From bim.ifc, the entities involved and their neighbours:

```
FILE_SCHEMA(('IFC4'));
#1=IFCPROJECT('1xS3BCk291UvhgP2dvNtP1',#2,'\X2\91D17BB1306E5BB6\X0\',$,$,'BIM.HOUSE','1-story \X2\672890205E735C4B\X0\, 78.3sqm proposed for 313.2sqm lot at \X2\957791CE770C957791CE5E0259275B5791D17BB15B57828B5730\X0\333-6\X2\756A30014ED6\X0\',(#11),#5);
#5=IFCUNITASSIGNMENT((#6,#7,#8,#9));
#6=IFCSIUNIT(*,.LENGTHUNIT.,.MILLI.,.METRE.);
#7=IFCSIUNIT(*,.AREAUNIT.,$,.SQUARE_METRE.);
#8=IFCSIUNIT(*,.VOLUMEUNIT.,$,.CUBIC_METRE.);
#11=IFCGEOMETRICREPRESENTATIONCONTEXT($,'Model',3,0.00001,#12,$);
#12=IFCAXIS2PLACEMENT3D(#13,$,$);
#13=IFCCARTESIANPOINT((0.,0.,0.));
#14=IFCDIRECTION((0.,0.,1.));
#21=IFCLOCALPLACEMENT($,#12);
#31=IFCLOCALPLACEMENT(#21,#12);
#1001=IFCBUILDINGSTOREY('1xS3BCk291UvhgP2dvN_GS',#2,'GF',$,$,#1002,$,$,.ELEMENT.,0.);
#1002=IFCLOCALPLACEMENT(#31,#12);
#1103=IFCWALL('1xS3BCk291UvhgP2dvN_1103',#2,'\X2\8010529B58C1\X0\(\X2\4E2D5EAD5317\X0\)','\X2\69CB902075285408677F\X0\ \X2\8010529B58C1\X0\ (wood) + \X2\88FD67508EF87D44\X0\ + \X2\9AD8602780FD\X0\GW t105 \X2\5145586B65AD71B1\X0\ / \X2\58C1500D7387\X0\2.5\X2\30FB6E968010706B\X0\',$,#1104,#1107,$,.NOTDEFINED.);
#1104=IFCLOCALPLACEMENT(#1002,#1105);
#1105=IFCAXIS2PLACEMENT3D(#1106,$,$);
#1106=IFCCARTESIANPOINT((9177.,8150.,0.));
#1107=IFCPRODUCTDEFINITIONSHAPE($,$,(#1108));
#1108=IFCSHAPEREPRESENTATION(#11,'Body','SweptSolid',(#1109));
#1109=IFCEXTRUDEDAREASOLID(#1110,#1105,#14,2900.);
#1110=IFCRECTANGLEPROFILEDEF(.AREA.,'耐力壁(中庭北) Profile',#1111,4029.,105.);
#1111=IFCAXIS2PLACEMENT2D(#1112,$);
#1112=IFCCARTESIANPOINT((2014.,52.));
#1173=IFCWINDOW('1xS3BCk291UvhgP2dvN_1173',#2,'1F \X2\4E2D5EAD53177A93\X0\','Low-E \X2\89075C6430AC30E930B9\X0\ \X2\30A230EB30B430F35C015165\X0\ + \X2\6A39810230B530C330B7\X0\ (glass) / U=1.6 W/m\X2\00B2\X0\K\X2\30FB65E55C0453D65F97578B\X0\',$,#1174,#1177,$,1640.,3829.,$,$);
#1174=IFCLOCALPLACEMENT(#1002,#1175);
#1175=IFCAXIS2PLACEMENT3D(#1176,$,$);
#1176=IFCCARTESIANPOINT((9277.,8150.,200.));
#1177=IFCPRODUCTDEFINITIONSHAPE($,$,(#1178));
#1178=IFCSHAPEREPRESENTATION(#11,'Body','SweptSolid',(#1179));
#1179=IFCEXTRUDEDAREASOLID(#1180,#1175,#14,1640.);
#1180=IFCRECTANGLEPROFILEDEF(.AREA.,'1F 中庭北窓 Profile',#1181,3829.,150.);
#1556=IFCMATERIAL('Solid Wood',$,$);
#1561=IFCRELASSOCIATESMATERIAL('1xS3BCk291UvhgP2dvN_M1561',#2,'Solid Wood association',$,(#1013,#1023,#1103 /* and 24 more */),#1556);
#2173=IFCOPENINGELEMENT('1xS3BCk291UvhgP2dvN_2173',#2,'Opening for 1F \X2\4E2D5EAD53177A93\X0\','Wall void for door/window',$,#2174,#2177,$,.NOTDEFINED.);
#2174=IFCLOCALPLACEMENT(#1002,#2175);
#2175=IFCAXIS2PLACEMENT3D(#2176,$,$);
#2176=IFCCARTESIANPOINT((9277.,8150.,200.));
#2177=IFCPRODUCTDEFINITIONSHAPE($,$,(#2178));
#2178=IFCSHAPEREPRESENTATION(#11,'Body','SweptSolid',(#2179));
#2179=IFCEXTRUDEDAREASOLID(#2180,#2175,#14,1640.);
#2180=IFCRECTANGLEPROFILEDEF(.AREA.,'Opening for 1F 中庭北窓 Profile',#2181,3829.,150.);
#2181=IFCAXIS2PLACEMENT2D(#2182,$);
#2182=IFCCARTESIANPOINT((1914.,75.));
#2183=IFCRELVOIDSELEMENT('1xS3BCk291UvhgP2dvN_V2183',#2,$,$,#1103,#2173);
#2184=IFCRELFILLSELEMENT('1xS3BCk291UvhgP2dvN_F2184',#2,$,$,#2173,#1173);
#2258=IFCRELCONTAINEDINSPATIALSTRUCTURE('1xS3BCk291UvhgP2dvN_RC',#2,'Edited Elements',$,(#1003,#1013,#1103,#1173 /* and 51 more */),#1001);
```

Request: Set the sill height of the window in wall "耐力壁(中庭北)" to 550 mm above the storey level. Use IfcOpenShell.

```python
import numpy as np
import ifcopenshell
import ifcopenshell.api.geometry
import ifcopenshell.geom
import ifcopenshell.util.element
import ifcopenshell.util.placement
import ifcopenshell.util.shape
import ifcopenshell.util.unit

model = ifcopenshell.open("bim.ifc")
unit_scale = ifcopenshell.util.unit.calculate_unit_scale(model)

window = model.by_guid("1xS3BCk291UvhgP2dvN_1173")
opening = window.FillsVoids[0].RelatingOpeningElement
storey = ifcopenshell.util.element.get_container(window, ifc_class="IfcBuildingStorey")
level = ifcopenshell.util.placement.get_local_placement(storey.ObjectPlacement)[2, 3]

# The opening's origin need not be at the sill, so measure its lowest point.
shape = ifcopenshell.geom.create_shape(ifcopenshell.geom.settings(), opening)
bottom = ifcopenshell.util.shape.get_shape_bottom_elevation(shape, shape.geometry) / unit_scale
dz = level + 550.0 - bottom

shift = np.array([0.0, 0.0, dz])
# The window is not placed relative to its opening, so move both.
for product in (opening, window):
    matrix = ifcopenshell.util.placement.get_local_placement(product.ObjectPlacement)
    matrix[:3, 3] += shift
    ifcopenshell.api.geometry.edit_object_placement(model, product=product, matrix=matrix, is_si=False)

print(f"moved by {dz * unit_scale:+.3f} m")

model.write("bim_updated.ifc")
```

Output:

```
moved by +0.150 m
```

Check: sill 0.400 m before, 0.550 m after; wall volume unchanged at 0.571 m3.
